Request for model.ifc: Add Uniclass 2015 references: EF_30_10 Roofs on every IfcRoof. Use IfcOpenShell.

First a look at what the model holds.

```python
import ifcopenshell

model = ifcopenshell.open("model.ifc")
print(model.schema)
print("classifications:", [c.Name for c in model.by_type("IfcClassification")])
for ifc_class in ("IfcDoor", "IfcRoof", "IfcStair", "IfcWall", "IfcWindow"):
    print(ifc_class, len(model.by_type(ifc_class)))
```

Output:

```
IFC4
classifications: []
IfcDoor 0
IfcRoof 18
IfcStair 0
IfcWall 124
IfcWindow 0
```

```python
import ifcopenshell
import ifcopenshell.api.classification

model = ifcopenshell.open("model.ifc")

system = ifcopenshell.api.classification.add_classification(model, classification="Uniclass 2015")

codes = {
    "IfcRoof": ("EF_30_10", "Roofs"),
}
for ifc_class, (code, name) in codes.items():
    products = model.by_type(ifc_class)
    ifcopenshell.api.classification.add_reference(
        model, products=products, classification=system, identification=code, name=name
    )
    print(code, len(products))

model.write("model_v2.ifc")
```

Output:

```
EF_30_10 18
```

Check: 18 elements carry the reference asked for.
